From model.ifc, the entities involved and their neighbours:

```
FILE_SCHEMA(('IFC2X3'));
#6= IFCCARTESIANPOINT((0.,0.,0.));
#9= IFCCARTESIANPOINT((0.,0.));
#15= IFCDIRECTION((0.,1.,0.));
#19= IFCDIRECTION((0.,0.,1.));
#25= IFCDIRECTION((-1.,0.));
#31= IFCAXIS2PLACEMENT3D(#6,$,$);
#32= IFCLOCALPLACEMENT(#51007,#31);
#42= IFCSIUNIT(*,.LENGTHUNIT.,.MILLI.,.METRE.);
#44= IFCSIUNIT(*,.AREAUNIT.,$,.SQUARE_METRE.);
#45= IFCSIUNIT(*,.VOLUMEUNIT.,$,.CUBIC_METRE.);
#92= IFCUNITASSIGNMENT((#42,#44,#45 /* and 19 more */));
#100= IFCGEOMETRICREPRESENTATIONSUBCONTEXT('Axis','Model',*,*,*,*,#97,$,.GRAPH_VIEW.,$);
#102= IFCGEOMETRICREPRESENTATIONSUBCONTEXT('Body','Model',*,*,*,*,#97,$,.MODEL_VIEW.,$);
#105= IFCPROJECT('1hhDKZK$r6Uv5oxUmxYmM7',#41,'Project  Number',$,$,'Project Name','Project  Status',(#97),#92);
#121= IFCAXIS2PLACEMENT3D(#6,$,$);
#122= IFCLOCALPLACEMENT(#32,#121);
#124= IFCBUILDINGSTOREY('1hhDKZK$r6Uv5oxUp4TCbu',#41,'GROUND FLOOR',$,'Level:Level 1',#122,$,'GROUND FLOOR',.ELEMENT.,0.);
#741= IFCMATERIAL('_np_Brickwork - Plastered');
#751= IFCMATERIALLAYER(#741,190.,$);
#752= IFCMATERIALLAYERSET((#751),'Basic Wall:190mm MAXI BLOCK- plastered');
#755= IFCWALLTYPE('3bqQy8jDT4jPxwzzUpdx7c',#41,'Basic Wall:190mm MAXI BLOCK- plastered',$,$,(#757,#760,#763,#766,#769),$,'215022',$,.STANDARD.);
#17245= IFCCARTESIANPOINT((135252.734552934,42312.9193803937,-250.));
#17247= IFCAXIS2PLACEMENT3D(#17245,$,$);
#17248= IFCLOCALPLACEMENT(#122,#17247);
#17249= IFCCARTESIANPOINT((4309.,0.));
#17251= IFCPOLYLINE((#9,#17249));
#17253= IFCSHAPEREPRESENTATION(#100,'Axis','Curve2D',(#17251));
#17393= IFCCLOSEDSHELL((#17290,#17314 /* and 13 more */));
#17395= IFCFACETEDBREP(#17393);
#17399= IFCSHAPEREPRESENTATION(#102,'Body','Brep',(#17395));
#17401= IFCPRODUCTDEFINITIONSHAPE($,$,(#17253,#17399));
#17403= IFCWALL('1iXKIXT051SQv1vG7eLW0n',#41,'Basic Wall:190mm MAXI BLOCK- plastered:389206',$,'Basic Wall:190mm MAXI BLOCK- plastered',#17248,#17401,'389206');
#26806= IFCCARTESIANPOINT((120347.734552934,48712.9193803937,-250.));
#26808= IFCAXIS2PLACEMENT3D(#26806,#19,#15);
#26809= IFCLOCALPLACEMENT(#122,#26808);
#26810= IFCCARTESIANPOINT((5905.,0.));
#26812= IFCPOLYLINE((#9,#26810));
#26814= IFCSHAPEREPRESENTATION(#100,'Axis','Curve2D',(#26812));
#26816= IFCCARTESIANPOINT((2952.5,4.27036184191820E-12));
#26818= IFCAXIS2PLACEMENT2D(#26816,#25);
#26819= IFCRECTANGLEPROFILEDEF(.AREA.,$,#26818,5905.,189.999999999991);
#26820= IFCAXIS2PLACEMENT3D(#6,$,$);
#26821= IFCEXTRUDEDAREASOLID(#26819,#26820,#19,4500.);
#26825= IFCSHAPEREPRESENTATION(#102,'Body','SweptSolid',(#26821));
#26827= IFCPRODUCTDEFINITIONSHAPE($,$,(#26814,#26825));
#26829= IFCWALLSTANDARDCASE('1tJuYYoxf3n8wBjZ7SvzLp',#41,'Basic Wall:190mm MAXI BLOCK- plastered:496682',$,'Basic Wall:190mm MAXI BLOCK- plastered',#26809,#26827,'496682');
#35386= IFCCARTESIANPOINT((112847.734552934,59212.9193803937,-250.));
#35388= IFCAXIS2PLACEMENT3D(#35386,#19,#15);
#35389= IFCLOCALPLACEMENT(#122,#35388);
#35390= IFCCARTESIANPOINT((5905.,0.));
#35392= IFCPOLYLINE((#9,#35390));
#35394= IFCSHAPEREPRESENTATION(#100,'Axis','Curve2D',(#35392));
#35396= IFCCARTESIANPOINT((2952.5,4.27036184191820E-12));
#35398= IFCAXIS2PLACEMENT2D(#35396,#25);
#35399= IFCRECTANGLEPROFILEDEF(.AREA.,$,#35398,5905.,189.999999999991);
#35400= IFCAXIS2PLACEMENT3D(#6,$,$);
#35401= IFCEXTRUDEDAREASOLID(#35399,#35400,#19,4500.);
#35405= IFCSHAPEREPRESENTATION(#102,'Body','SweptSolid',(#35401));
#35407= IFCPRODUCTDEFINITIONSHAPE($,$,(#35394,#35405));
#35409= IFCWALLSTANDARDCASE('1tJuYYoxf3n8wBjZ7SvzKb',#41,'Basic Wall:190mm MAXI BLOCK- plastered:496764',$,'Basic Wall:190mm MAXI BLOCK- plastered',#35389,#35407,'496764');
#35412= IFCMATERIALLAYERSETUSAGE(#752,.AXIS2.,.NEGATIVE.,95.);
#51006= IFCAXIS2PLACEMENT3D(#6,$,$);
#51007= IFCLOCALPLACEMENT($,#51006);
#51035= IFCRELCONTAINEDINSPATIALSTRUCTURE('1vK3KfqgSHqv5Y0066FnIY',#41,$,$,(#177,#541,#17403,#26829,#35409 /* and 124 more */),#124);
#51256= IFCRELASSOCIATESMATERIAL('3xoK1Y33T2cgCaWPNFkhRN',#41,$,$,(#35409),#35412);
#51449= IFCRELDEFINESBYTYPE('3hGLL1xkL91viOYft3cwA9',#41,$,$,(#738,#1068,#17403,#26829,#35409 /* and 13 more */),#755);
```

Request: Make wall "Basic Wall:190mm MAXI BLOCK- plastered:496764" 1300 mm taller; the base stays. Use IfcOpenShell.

```python
import ifcopenshell
import ifcopenshell.geom
import ifcopenshell.util.representation
import ifcopenshell.util.shape
import ifcopenshell.util.unit

model = ifcopenshell.open("model.ifc")
unit_scale = ifcopenshell.util.unit.calculate_unit_scale(model)
settings = ifcopenshell.geom.settings()


def volume(element):
    """Net volume in cubic metres, openings subtracted."""
    shape = ifcopenshell.geom.create_shape(settings, element)
    return ifcopenshell.util.shape.get_volume(shape.geometry)


wall = model.by_guid("1tJuYYoxf3n8wBjZ7SvzKb")
before = volume(wall)

body = ifcopenshell.util.representation.get_representation(wall, "Model", "Body")
solid = body.Items[0]
old_height = solid.Depth
solid.Depth += 1.3 / unit_scale
after = volume(wall)

print(f"height {old_height:g} -> {solid.Depth:g}, volume {before:.3f} -> {after:.3f} m3")

model.write("model_updated.ifc")
```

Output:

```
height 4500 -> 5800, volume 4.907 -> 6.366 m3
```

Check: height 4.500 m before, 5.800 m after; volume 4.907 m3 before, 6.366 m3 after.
